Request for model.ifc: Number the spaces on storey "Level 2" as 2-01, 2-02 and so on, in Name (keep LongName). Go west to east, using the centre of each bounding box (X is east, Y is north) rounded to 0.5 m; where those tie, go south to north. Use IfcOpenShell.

First a look at what the model holds.

```python
import ifcopenshell
import ifcopenshell.util.element
import ifcopenshell.util.placement

model = ifcopenshell.open("model.ifc")
print(model.schema)
storey = next(s for s in model.by_type("IfcBuildingStorey") if s.Name == "Level 2")
spaces = [e for e in ifcopenshell.util.element.get_decomposition(storey) if e.is_a("IfcSpace")]
for e in sorted(spaces, key=lambda e: e.id()):
    origin = ifcopenshell.util.placement.get_local_placement(e.ObjectPlacement)[:3, 3]
    print(e.id(), e.Name, e.LongName, origin.round(2) + 0.0, sep=" | ")
```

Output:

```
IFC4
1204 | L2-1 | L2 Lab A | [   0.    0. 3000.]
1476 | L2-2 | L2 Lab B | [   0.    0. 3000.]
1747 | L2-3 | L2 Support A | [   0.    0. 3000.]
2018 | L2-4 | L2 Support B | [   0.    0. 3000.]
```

```python
import ifcopenshell
import ifcopenshell.geom
import ifcopenshell.util.element
import ifcopenshell.util.shape

model = ifcopenshell.open("model.ifc")
settings = ifcopenshell.geom.settings()
settings.set("use-world-coords", True)


def centre(element):
    shape = ifcopenshell.geom.create_shape(settings, element)
    return ifcopenshell.util.shape.get_bbox_centroid(shape.geometry)


storey = next(s for s in model.by_type("IfcBuildingStorey") if s.Name == "Level 2")
spaces = [e for e in ifcopenshell.util.element.get_decomposition(storey) if e.is_a("IfcSpace")]

# Insertion points can sit at a corner or the storey origin, so sort by the geometry (in metres).
centres = {e: centre(e) for e in spaces}
spaces.sort(key=lambda e: (round(centres[e][0] / 0.5), centres[e][1]))

for i, e in enumerate(spaces, start=1):
    number = f"2-{i:02d}"
    e.Name = number
    print(e.id(), number)

model.write("model_v2.ifc")
```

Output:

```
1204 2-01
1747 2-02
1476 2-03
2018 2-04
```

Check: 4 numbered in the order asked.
